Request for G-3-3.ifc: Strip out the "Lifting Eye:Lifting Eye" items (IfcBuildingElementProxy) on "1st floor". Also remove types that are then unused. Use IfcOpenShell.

First a look at what the model holds.

```python
import ifcopenshell
import ifcopenshell.util.element

model = ifcopenshell.open("G-3-3.ifc")
print(model.schema)
storey = next(s for s in model.by_type("IfcBuildingStorey") if s.Name == "1st floor")
proxies = [e for e in ifcopenshell.util.element.get_decomposition(storey) if e.is_a("IfcBuildingElementProxy")]
seen = {}
for e in proxies:
    element_type = ifcopenshell.util.element.get_type(e)
    name = element_type.Name if element_type not in (None, e) else None
    seen[name] = seen.get(name, 0) + 1
for name, count in sorted(seen.items(), key=str):
    print(count, "x", name)
```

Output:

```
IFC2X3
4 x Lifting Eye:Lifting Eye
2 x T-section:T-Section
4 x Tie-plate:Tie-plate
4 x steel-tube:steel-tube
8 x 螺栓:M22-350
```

```python
import ifcopenshell
import ifcopenshell.api.root
import ifcopenshell.util.element

model = ifcopenshell.open("G-3-3.ifc")

storey = next(s for s in model.by_type("IfcBuildingStorey") if s.Name == "1st floor")
proxies = [e for e in ifcopenshell.util.element.get_decomposition(storey) if e.is_a("IfcBuildingElementProxy")]
targets = [e for e in proxies if (t := ifcopenshell.util.element.get_type(e)) not in (None, e) and t.Name == "Lifting Eye:Lifting Eye"]
types = {ifcopenshell.util.element.get_type(e) for e in targets} - {None, *targets}

for e in targets:
    ifcopenshell.api.root.remove_product(model, product=e)
print(len(targets), "removed")

unused = [t for t in types if not ifcopenshell.util.element.get_types(t)]
for t in unused:
    ifcopenshell.api.root.remove_product(model, product=t)
print(len(unused), "unused types removed")

model.write("G-3-3_v2.ifc")
```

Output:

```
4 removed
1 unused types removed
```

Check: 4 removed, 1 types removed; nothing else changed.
